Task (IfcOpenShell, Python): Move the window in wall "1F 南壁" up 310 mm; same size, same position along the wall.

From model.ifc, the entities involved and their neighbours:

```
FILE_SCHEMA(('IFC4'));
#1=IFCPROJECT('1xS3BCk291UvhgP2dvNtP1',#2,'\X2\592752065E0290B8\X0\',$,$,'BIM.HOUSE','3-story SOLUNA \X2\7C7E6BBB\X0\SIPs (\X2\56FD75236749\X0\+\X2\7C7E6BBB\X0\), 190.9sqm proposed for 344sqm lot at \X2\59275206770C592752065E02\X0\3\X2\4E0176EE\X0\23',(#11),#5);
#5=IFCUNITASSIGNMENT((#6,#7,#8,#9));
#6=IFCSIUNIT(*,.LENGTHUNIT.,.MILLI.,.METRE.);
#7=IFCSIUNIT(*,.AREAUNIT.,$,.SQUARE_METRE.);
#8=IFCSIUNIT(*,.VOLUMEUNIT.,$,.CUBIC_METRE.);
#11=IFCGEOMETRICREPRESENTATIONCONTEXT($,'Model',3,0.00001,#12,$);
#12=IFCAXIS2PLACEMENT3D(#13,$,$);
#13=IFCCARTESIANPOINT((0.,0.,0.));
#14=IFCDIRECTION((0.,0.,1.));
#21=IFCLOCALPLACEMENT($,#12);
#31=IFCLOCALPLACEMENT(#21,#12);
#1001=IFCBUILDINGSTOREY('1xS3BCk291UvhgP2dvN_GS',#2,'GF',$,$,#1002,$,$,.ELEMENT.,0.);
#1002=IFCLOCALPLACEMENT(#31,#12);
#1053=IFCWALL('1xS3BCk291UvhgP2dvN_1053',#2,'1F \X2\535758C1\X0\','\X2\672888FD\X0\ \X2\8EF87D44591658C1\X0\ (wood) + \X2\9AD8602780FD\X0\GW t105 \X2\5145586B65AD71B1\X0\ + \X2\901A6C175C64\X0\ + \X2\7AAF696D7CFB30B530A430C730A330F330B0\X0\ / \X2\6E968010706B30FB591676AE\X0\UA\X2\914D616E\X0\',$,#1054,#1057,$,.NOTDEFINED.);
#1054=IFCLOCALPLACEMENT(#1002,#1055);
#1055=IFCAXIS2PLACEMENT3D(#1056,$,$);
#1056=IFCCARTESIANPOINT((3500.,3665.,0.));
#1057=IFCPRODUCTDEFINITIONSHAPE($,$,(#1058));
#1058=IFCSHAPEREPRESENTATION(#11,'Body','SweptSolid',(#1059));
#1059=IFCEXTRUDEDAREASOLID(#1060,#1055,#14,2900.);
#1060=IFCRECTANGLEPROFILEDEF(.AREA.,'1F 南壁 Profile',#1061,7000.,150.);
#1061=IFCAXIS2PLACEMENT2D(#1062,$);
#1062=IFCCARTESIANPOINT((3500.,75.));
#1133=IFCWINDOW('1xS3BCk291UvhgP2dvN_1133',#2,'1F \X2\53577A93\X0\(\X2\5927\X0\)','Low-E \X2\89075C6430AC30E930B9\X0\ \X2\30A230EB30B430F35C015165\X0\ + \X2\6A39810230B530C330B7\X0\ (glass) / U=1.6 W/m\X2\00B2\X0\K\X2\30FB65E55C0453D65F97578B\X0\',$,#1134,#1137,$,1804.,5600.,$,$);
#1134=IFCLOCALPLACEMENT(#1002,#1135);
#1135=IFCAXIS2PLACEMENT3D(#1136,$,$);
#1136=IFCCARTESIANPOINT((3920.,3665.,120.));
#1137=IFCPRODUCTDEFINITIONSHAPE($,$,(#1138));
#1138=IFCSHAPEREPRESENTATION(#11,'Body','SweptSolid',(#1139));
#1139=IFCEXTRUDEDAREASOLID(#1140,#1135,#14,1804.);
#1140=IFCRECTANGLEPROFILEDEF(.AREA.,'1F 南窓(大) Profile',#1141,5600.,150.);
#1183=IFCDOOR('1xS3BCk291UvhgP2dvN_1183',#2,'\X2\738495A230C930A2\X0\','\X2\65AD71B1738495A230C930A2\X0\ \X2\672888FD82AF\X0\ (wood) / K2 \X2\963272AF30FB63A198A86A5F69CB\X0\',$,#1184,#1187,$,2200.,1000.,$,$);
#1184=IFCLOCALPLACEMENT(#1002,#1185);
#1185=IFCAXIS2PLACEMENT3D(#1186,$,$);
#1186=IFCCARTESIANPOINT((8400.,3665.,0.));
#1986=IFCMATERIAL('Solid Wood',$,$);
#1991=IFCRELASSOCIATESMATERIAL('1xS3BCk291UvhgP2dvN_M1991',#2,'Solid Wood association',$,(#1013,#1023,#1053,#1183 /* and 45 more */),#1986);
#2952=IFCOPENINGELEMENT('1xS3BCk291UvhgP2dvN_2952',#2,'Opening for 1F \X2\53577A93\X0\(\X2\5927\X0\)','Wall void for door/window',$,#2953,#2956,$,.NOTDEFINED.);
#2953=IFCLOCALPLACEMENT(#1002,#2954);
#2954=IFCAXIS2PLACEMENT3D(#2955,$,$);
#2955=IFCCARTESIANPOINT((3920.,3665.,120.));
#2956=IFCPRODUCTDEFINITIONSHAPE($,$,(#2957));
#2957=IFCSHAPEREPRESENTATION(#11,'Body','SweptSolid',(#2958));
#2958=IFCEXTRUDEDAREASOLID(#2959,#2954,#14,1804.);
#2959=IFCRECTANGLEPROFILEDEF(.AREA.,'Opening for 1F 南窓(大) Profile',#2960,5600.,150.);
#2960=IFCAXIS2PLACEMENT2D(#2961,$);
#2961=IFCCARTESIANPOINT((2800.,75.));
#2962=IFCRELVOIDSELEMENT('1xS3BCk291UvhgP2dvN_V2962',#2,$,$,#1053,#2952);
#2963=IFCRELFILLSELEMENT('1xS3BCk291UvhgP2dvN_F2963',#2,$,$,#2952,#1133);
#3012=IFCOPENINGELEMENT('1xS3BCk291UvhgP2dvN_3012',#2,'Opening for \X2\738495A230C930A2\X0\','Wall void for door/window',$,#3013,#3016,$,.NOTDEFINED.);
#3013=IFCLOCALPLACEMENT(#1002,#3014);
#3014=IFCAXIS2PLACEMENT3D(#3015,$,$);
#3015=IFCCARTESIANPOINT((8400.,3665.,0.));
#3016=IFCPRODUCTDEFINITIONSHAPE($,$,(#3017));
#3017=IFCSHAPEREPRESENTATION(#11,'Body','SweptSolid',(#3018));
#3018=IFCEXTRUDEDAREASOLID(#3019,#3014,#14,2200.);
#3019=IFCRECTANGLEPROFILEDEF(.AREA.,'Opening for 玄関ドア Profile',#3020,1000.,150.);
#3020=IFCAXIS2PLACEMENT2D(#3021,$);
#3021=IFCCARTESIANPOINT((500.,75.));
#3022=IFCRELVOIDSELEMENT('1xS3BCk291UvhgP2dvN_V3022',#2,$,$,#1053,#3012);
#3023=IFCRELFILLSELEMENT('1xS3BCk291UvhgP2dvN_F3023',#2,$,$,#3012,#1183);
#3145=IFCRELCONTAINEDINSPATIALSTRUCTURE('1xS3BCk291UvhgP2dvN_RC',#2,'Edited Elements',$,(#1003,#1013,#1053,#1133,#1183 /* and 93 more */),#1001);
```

```python
import numpy as np
import ifcopenshell
import ifcopenshell.api.geometry
import ifcopenshell.util.placement
import ifcopenshell.util.unit

model = ifcopenshell.open("model.ifc")
unit_scale = ifcopenshell.util.unit.calculate_unit_scale(model)

window = model.by_id(1133)
opening = window.FillsVoids[0].RelatingOpeningElement
dz = 0.31 / unit_scale

shift = np.array([0.0, 0.0, dz])
# The window is not placed relative to its opening, so move both.
for product in (opening, window):
    matrix = ifcopenshell.util.placement.get_local_placement(product.ObjectPlacement)
    matrix[:3, 3] += shift
    ifcopenshell.api.geometry.edit_object_placement(model, product=product, matrix=matrix, is_si=False)

print(f"moved by {dz * unit_scale:+.3f} m")

model.write("model_v2.ifc")
```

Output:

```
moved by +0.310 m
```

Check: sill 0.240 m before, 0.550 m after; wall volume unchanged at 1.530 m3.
